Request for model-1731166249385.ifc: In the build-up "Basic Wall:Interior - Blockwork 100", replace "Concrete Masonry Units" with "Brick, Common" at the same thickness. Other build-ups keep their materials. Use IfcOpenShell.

First a look at what the model holds.

```python
import ifcopenshell
import ifcopenshell.util.element

model = ifcopenshell.open("model-1731166249385.ifc")
print(model.schema)
for layer_set in model.by_type("IfcMaterialLayerSet"):
    if layer_set.LayerSetName == "Basic Wall:Interior - Blockwork 100":
        for layer in layer_set.MaterialLayers:
            print(layer.id(), layer.Material and layer.Material.Name, layer.LayerThickness, sep=" | ")
        print(len(ifcopenshell.util.element.get_elements_by_material(model, layer_set)), "elements and types use it")
print(sorted(m.Name for m in model.by_type("IfcMaterial") if m.Name)[:60])
```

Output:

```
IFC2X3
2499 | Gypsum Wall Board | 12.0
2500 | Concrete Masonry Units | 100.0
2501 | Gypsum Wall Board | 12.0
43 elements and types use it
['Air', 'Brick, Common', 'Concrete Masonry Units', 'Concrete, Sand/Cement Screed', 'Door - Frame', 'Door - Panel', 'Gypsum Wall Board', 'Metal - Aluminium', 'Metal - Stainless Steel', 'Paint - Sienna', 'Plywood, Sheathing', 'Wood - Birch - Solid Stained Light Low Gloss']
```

```python
import ifcopenshell
import ifcopenshell.api.material

model = ifcopenshell.open("model-1731166249385.ifc")

layer_set = next(s for s in model.by_type("IfcMaterialLayerSet") if s.LayerSetName == "Basic Wall:Interior - Blockwork 100")
layer = next(l for l in layer_set.MaterialLayers if l.Material and l.Material.Name == "Concrete Masonry Units")
material = next(m for m in model.by_type("IfcMaterial") if m.Name == "Brick, Common")

# Point this one layer at the other material; renaming the old one would change it everywhere.
ifcopenshell.api.material.edit_layer(model, layer=layer, attributes={}, material=material)

print([l.Material.Name if l.Material else None for l in layer_set.MaterialLayers])

model.write("model-1731166249385_v2.ifc")
```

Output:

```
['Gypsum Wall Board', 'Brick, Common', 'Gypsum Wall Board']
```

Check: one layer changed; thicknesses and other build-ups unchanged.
